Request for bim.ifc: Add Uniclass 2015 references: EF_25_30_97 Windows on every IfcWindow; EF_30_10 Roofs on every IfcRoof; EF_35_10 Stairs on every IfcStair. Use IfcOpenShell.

First a look at what the model holds.

```python
import ifcopenshell

model = ifcopenshell.open("bim.ifc")
print(model.schema)
print("classifications:", [c.Name for c in model.by_type("IfcClassification")])
for ifc_class in ("IfcDoor", "IfcRoof", "IfcStair", "IfcWall", "IfcWindow"):
    print(ifc_class, len(model.by_type(ifc_class)))
```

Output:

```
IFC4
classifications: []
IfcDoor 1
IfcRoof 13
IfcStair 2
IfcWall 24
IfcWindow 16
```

```python
import ifcopenshell
import ifcopenshell.api.classification

model = ifcopenshell.open("bim.ifc")

system = ifcopenshell.api.classification.add_classification(model, classification="Uniclass 2015")

codes = {
    "IfcWindow": ("EF_25_30_97", "Windows"),
    "IfcRoof": ("EF_30_10", "Roofs"),
    "IfcStair": ("EF_35_10", "Stairs"),
}
for ifc_class, (code, name) in codes.items():
    products = model.by_type(ifc_class)
    ifcopenshell.api.classification.add_reference(
        model, products=products, classification=system, identification=code, name=name
    )
    print(code, len(products))

model.write("bim_edited.ifc")
```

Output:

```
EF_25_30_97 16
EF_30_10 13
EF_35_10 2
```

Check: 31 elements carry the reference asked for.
